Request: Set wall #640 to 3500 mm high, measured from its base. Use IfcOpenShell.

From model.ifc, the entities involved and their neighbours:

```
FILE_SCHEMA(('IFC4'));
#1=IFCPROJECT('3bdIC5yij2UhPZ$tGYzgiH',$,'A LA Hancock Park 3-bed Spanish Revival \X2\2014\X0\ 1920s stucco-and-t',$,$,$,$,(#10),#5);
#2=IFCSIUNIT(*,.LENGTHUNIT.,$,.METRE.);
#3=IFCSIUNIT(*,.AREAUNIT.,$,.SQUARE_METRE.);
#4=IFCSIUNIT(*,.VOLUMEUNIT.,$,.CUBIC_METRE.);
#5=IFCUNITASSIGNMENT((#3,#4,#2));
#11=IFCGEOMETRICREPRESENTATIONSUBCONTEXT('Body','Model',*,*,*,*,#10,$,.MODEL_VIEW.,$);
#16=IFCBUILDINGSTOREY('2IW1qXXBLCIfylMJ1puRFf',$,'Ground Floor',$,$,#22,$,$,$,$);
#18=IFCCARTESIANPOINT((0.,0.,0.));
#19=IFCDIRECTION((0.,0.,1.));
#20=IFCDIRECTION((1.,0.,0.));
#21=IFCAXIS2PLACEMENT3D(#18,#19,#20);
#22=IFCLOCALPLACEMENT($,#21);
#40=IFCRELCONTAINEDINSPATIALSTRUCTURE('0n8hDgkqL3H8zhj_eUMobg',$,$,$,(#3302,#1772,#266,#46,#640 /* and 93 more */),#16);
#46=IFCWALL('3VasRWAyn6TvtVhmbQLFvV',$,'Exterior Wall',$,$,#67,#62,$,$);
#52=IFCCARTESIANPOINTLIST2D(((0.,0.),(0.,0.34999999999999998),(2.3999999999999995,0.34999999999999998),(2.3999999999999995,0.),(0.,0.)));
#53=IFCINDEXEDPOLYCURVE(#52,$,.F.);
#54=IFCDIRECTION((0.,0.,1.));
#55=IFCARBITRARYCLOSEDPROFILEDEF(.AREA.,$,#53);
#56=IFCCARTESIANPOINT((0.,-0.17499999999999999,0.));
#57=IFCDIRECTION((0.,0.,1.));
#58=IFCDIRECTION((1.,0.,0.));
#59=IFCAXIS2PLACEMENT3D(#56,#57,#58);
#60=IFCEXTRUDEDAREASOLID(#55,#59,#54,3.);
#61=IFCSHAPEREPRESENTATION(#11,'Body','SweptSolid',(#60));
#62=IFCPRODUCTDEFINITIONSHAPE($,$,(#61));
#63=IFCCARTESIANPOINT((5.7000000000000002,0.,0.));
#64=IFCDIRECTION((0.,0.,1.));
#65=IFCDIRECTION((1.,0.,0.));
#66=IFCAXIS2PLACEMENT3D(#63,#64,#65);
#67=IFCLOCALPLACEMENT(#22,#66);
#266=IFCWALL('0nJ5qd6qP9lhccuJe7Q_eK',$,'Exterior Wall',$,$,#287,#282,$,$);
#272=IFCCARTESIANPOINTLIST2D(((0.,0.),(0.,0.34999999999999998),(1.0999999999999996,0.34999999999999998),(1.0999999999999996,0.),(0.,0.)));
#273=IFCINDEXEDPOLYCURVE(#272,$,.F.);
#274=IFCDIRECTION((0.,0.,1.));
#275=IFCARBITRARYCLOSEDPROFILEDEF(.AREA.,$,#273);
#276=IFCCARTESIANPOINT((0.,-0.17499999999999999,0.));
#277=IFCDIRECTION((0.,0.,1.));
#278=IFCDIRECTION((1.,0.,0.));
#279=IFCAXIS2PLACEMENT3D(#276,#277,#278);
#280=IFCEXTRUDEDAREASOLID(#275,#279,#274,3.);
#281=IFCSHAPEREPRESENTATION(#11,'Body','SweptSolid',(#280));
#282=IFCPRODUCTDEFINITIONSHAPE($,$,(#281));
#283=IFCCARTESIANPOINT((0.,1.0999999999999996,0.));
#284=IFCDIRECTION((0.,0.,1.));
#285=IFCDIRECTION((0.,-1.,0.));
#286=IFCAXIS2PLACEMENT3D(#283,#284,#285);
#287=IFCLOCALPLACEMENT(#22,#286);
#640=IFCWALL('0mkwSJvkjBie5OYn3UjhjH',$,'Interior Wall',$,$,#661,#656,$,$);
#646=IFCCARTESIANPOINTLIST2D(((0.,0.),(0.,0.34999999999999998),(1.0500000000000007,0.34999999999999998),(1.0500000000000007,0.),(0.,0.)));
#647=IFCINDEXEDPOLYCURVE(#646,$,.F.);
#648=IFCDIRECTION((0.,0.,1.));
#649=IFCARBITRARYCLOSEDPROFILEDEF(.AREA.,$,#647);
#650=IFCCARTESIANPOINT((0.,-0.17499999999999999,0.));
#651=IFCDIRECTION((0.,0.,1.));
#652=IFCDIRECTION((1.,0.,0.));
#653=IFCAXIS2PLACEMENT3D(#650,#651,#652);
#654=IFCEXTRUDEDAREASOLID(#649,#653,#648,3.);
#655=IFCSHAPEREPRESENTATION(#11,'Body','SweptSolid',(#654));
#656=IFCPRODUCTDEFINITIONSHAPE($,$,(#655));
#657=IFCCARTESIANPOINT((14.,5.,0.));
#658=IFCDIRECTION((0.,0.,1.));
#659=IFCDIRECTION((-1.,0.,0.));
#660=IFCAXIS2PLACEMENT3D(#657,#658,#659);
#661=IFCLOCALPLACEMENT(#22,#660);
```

```python
import ifcopenshell
import ifcopenshell.geom
import ifcopenshell.util.representation
import ifcopenshell.util.shape

model = ifcopenshell.open("model.ifc")
settings = ifcopenshell.geom.settings()


def volume(element):
    """Net volume in cubic metres, openings subtracted."""
    shape = ifcopenshell.geom.create_shape(settings, element)
    return ifcopenshell.util.shape.get_volume(shape.geometry)


wall = model.by_guid("0mkwSJvkjBie5OYn3UjhjH")
before = volume(wall)

body = ifcopenshell.util.representation.get_representation(wall, "Model", "Body")
solid = body.Items[0]
old_height = solid.Depth
solid.Depth = 3.5
after = volume(wall)

print(f"height {old_height:g} -> {solid.Depth:g}, volume {before:.3f} -> {after:.3f} m3")

model.write("model_updated.ifc")
```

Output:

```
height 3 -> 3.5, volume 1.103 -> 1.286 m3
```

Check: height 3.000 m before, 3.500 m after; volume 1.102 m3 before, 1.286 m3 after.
